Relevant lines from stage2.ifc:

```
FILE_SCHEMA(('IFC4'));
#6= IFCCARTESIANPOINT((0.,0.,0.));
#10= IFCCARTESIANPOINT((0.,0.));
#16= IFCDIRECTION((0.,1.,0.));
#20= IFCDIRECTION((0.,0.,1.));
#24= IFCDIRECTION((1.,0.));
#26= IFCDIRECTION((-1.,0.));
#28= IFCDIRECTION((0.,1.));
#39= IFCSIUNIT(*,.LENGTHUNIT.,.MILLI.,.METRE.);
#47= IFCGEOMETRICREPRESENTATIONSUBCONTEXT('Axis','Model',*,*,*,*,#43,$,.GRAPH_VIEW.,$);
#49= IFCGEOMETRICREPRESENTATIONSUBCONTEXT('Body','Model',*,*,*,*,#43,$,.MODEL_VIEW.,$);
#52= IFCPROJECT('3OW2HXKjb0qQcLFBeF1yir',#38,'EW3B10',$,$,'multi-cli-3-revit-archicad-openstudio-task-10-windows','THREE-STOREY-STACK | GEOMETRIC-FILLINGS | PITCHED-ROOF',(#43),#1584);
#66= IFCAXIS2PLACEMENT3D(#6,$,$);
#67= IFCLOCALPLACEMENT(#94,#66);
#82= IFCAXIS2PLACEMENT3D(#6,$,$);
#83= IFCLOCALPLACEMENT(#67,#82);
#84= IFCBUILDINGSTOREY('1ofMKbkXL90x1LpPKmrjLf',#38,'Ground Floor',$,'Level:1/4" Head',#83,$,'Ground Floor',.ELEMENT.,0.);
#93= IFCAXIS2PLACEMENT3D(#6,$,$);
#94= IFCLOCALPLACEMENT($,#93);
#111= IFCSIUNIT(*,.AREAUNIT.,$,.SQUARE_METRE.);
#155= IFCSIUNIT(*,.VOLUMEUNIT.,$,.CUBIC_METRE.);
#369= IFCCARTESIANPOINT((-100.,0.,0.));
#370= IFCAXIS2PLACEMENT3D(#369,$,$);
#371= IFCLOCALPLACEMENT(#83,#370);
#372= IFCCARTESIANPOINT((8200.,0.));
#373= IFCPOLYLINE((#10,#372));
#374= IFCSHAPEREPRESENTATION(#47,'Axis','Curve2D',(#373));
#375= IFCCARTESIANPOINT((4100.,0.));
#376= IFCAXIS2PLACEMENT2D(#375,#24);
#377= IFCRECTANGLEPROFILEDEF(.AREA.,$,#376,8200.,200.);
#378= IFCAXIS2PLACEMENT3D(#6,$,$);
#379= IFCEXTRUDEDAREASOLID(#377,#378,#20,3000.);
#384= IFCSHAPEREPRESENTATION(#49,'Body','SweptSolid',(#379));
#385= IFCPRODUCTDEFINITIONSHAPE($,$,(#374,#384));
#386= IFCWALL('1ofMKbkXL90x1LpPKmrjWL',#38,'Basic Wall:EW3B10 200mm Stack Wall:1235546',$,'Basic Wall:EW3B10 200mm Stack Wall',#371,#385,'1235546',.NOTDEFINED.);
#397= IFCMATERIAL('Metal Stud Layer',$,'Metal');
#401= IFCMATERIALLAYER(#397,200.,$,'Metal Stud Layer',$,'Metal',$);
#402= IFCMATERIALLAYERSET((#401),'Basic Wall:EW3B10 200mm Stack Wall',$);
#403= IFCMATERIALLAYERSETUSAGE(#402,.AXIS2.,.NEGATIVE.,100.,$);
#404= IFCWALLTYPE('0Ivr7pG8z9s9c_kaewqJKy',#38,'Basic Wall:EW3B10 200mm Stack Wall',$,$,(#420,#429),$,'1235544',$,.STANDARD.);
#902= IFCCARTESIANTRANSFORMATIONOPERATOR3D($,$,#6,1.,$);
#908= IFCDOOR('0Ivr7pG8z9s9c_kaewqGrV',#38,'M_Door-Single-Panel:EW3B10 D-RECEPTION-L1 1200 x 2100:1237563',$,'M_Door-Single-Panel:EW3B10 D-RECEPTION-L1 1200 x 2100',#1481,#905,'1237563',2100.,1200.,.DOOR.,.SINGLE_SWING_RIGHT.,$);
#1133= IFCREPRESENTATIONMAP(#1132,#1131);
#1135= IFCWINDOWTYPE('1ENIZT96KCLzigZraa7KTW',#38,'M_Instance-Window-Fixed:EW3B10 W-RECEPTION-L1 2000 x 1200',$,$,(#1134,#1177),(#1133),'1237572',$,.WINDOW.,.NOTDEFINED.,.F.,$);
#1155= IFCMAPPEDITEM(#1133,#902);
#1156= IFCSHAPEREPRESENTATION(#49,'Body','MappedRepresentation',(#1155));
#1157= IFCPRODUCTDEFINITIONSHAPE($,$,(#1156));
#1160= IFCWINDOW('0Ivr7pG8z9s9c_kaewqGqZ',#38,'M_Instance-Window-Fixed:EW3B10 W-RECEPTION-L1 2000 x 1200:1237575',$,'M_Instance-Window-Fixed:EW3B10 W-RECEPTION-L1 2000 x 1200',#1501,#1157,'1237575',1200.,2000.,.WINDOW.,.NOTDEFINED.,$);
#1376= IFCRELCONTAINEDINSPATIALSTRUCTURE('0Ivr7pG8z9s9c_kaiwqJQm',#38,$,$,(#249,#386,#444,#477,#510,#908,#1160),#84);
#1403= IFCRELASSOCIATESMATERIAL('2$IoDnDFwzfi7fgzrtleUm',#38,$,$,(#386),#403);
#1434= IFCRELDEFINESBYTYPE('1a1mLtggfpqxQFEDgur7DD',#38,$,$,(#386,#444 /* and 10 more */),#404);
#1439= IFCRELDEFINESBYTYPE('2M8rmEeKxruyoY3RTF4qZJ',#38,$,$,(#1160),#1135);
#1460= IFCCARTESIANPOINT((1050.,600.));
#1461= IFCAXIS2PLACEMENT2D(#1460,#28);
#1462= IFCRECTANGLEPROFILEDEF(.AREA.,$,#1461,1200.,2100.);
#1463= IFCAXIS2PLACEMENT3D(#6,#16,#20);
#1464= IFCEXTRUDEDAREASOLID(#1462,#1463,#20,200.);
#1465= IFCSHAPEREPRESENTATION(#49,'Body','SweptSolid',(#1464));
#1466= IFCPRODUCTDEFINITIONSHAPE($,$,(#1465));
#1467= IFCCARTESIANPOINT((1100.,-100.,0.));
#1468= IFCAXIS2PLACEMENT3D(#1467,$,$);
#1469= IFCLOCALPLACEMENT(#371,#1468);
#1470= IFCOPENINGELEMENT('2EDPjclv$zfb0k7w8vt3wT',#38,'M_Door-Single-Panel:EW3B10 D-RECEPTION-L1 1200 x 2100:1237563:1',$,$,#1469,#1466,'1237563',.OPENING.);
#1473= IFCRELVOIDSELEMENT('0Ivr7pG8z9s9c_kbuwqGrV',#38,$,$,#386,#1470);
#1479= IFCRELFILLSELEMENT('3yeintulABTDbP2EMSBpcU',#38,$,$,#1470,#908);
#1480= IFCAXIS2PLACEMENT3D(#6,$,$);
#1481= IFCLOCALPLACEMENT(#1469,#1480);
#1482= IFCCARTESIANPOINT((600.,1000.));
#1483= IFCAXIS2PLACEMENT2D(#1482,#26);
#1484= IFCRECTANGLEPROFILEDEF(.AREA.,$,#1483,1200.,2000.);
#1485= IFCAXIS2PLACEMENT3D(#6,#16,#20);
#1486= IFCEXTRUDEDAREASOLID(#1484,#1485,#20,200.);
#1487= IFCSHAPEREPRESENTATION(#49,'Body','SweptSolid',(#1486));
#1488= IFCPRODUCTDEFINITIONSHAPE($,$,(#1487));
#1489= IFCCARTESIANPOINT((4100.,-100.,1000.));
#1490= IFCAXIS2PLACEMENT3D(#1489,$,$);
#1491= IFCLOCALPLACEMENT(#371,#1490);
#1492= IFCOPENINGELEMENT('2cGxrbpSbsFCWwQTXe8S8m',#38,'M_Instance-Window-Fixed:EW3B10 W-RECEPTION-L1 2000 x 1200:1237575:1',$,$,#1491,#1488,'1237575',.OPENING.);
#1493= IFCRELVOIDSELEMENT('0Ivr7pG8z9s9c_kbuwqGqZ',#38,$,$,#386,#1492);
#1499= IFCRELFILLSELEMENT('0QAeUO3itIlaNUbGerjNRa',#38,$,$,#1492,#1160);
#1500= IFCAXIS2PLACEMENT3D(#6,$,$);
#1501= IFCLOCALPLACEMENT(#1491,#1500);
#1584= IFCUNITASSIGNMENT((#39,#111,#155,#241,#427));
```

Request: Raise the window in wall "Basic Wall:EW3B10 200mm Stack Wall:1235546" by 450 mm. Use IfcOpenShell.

```python
import numpy as np
import ifcopenshell
import ifcopenshell.api.geometry
import ifcopenshell.util.placement
import ifcopenshell.util.unit

model = ifcopenshell.open("stage2.ifc")
unit_scale = ifcopenshell.util.unit.calculate_unit_scale(model)

window = model.by_id(1160)
opening = window.FillsVoids[0].RelatingOpeningElement
dz = 450.0

shift = np.array([0.0, 0.0, dz])
# The window is placed relative to its opening, so it follows when the opening moves.
matrix = ifcopenshell.util.placement.get_local_placement(opening.ObjectPlacement)
matrix[:3, 3] += shift
ifcopenshell.api.geometry.edit_object_placement(
    model, product=opening, matrix=matrix, is_si=False, should_transform_children=True
)

print(f"moved by {dz * unit_scale:+.3f} m")

model.write("stage2-out.ifc")
```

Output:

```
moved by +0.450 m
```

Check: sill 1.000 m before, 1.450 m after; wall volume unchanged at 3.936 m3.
